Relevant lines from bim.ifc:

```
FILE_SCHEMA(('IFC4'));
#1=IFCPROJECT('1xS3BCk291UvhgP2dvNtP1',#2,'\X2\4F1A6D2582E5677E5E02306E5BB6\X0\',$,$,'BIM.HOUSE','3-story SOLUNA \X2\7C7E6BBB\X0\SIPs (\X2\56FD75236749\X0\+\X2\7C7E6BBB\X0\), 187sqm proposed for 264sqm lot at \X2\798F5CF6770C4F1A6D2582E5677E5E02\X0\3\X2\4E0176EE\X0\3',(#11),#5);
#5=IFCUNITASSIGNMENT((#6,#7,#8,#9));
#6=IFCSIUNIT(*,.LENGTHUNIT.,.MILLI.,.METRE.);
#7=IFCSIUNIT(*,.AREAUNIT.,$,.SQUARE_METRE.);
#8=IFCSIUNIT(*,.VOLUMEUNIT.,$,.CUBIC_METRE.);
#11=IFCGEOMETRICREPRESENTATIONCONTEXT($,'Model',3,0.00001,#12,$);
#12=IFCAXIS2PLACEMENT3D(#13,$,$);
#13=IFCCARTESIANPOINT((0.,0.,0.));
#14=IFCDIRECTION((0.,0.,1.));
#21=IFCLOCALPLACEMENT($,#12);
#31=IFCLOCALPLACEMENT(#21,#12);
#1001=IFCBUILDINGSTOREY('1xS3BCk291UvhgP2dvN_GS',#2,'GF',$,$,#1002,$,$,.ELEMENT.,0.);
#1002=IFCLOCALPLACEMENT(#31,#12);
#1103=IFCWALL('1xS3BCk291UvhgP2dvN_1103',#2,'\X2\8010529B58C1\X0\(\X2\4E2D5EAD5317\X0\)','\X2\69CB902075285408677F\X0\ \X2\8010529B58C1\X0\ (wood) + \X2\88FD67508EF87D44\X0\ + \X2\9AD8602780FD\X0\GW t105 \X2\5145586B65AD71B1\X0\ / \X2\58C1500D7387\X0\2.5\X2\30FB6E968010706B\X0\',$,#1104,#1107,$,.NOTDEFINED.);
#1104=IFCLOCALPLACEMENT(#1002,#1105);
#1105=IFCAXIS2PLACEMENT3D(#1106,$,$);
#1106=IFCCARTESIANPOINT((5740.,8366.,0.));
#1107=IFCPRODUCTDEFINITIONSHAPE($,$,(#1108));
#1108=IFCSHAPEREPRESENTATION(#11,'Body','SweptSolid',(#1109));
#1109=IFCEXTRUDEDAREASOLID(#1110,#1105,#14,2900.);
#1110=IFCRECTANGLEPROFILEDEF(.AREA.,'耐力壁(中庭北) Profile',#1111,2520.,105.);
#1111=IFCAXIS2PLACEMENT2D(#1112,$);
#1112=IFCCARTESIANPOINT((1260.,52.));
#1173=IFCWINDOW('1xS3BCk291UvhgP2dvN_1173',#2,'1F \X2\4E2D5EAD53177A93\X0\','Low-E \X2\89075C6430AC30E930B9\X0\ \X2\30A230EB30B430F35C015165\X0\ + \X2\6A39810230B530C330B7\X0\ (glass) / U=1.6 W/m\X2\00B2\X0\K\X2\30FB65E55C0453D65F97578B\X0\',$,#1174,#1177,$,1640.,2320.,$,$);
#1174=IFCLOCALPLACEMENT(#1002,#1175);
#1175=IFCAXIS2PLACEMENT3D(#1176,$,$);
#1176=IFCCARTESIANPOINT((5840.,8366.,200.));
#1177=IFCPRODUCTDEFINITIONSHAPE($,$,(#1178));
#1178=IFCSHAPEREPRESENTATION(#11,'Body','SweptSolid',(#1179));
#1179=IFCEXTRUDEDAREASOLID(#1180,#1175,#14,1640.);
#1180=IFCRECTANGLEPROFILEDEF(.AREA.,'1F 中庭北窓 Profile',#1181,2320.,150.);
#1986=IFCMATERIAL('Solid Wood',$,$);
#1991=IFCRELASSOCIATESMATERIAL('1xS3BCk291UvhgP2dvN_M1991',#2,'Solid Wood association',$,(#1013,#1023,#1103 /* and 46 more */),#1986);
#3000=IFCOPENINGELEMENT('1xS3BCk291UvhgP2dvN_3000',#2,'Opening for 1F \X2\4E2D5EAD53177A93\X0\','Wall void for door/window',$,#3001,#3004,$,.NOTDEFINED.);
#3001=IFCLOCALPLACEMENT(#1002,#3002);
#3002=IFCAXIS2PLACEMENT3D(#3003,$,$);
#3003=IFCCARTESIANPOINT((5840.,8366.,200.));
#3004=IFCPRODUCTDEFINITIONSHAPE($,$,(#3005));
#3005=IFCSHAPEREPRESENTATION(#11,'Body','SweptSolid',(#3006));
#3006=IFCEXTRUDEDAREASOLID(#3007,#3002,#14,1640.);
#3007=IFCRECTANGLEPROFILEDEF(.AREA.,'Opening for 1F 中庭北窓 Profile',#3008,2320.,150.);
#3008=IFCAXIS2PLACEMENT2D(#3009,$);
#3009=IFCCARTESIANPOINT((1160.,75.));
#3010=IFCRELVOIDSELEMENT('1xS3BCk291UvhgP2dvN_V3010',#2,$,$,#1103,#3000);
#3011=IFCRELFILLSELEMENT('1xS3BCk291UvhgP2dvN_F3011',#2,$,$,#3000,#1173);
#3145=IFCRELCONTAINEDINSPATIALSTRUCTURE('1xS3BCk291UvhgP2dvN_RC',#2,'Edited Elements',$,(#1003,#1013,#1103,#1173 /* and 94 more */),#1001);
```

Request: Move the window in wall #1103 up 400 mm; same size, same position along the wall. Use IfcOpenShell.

```python
import numpy as np
import ifcopenshell
import ifcopenshell.api.geometry
import ifcopenshell.util.placement
import ifcopenshell.util.unit

model = ifcopenshell.open("bim.ifc")
unit_scale = ifcopenshell.util.unit.calculate_unit_scale(model)

window = model.by_guid("1xS3BCk291UvhgP2dvN_1173")
opening = window.FillsVoids[0].RelatingOpeningElement
dz = 400.0

shift = np.array([0.0, 0.0, dz])
# The window is not placed relative to its opening, so move both.
for product in (opening, window):
    matrix = ifcopenshell.util.placement.get_local_placement(product.ObjectPlacement)
    matrix[:3, 3] += shift
    ifcopenshell.api.geometry.edit_object_placement(model, product=product, matrix=matrix, is_si=False)

print(f"moved by {dz * unit_scale:+.3f} m")

model.write("bim-out.ifc")
```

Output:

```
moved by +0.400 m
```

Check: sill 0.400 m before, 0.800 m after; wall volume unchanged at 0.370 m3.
